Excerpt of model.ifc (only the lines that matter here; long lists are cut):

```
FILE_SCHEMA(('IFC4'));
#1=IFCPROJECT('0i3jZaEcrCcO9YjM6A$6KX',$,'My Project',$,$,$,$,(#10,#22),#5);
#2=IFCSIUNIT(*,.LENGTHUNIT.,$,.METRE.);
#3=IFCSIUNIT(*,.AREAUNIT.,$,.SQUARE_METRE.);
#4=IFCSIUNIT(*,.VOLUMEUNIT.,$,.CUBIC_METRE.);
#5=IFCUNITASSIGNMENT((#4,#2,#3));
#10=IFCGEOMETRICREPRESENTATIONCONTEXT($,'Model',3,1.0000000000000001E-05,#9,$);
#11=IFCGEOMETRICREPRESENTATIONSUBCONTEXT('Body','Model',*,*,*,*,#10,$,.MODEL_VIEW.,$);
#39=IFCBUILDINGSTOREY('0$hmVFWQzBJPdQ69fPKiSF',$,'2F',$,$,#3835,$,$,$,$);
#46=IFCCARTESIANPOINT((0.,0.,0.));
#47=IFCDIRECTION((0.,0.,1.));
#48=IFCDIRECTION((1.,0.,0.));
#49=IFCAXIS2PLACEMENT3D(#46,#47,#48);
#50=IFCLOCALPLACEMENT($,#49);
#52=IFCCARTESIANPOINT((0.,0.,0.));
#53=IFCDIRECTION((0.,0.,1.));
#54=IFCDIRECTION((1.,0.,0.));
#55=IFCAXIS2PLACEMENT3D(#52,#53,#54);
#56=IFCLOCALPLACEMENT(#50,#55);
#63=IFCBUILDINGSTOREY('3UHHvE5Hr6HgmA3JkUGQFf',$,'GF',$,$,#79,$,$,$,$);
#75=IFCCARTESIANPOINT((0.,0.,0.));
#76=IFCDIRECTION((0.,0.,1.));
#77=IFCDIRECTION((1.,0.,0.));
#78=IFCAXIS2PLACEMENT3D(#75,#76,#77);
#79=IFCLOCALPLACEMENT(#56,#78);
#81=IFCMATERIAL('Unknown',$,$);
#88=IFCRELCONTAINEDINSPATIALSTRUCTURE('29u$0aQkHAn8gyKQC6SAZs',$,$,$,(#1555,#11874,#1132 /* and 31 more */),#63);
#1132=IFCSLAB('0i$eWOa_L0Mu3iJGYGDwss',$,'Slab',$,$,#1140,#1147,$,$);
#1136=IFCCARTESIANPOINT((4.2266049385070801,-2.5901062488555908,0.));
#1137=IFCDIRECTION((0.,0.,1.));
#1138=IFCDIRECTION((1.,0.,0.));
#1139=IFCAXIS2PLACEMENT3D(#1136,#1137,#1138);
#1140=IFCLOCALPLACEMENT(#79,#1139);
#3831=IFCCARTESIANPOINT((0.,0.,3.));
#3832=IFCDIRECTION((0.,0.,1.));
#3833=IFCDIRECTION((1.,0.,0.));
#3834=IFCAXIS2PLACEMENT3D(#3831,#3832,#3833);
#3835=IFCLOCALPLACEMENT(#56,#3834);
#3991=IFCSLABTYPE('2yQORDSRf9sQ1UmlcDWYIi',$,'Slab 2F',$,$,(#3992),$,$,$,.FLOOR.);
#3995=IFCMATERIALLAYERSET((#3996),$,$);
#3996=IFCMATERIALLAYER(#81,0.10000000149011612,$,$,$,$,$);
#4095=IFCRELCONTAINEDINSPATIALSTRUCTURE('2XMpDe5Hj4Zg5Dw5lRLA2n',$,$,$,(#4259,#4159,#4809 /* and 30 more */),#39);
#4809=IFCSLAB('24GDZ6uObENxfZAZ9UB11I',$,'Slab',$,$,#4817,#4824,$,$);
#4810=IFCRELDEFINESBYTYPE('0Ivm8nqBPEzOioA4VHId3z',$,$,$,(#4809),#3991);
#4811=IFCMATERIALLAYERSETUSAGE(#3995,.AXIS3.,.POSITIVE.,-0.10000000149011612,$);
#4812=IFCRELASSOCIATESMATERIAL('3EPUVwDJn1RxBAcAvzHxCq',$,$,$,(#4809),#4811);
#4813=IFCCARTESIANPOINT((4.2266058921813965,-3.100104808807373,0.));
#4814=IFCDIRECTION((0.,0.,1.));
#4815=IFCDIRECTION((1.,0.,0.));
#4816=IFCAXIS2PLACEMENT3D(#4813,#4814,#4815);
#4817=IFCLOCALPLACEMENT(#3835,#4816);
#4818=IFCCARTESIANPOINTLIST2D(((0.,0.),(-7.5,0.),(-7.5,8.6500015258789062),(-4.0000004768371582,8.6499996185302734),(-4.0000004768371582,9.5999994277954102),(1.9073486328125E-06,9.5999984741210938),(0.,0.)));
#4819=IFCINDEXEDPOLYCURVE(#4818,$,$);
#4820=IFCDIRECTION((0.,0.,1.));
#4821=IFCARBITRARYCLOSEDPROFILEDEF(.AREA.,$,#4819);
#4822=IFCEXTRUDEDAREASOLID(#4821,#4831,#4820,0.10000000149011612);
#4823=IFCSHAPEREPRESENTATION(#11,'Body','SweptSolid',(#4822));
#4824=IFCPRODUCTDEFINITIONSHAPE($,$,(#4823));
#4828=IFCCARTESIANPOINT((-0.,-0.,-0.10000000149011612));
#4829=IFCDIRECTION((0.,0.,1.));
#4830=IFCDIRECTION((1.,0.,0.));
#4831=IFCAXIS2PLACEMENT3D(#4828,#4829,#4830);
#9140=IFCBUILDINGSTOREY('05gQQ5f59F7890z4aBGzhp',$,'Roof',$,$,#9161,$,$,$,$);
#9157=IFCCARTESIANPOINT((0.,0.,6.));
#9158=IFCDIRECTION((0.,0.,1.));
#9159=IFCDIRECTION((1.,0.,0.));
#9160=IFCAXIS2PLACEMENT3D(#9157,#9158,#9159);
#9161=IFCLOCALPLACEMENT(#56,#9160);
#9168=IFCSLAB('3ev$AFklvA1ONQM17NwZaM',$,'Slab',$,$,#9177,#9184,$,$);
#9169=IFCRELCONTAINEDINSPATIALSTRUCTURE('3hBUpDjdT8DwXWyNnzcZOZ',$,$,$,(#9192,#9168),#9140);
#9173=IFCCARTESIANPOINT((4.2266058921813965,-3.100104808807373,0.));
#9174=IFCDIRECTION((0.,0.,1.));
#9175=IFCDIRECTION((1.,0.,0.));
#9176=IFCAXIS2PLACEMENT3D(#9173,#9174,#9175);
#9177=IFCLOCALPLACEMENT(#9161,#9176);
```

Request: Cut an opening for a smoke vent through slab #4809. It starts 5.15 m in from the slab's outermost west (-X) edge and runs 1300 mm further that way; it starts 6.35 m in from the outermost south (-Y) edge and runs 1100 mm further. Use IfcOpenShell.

```python
import numpy as np
import ifcopenshell
import ifcopenshell.api.feature
import ifcopenshell.api.geometry
import ifcopenshell.api.root
import ifcopenshell.geom
import ifcopenshell.util.placement
import ifcopenshell.util.representation
import ifcopenshell.util.shape
import ifcopenshell.util.unit

model = ifcopenshell.open("model.ifc")
unit_scale = ifcopenshell.util.unit.calculate_unit_scale(model)
settings = ifcopenshell.geom.settings()


def volume(element):
    """Net volume in cubic metres, openings subtracted."""
    shape = ifcopenshell.geom.create_shape(settings, element)
    return ifcopenshell.util.shape.get_volume(shape.geometry)


slab = model.by_guid("24GDZ6uObENxfZAZ9UB11I")
before = volume(slab)

# Extent in the slab's own axes, in metres. The edges named are its -X and -Y sides.
slab_shape = ifcopenshell.geom.create_shape(settings, slab)
vertices = ifcopenshell.util.shape.get_vertices(slab_shape.geometry)
x_min, y_min, bottom = vertices.min(axis=0)
top = vertices[:, 2].max()

opening = ifcopenshell.api.root.create_entity(model, ifc_class="IfcOpeningElement", name="Smoke vent opening", predefined_type="OPENING")
context = ifcopenshell.util.representation.get_context(model, "Model", "Body", "MODEL_VIEW")
width, depth = 1.3, 1.1
outline = [(0.0, 0.0), (width, 0.0), (width, depth), (0.0, depth), (0.0, 0.0)]
# Overshoot both faces by 50 mm so the cut is clean.
shape = ifcopenshell.api.geometry.add_slab_representation(
    model, context=context, depth=top - bottom + 0.1, polyline=outline
)
ifcopenshell.api.geometry.assign_representation(model, product=opening, representation=shape)

matrix = ifcopenshell.util.placement.get_local_placement(slab.ObjectPlacement)
matrix[:, 3] = matrix @ np.append(np.array([x_min + 5.15, y_min + 6.35, bottom - 0.05]) / unit_scale, 1.0)
ifcopenshell.api.geometry.edit_object_placement(model, product=opening, matrix=matrix, is_si=False)
ifcopenshell.api.feature.add_feature(model, feature=opening, element=slab)

after = volume(slab)

print(f"slab volume {before:.3f} -> {after:.3f} m3")

model.write("model_edited.ifc")
```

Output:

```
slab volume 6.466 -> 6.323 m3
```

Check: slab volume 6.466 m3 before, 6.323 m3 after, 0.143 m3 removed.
